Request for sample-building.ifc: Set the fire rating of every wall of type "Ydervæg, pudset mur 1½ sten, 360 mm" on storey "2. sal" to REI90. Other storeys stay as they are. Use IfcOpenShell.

First a look at what the model holds.

```python
import ifcopenshell
import ifcopenshell.util.element

model = ifcopenshell.open("sample-building.ifc")
print(model.schema)
storey = next(s for s in model.by_type("IfcBuildingStorey") if s.Name == "2. sal")
walls = [e for e in ifcopenshell.util.element.get_decomposition(storey) if e.is_a("IfcWall")]
seen = {}
for e in walls:
    element_type = ifcopenshell.util.element.get_type(e)
    key = (element_type.Name if element_type != e and element_type else None, ifcopenshell.util.element.get_pset(e, "Pset_WallCommon", "FireRating"))
    seen[key] = seen.get(key, 0) + 1
for (name, value), count in sorted(seen.items(), key=str):
    print(count, "x", name, "|", value)
```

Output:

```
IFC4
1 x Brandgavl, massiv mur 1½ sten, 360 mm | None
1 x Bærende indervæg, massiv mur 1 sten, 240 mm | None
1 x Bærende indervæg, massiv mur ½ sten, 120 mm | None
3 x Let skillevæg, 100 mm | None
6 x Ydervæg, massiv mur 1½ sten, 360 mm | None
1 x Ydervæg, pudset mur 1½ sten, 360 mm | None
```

```python
import ifcopenshell
import ifcopenshell.api.pset
import ifcopenshell.util.element

model = ifcopenshell.open("sample-building.ifc")

storey = next(s for s in model.by_type("IfcBuildingStorey") if s.Name == "2. sal")
walls = [e for e in ifcopenshell.util.element.get_decomposition(storey) if e.is_a("IfcWall")]

count = 0
for e in walls:
    element_type = ifcopenshell.util.element.get_type(e)
    if element_type in (None, e) or element_type.Name != "Ydervæg, pudset mur 1½ sten, 360 mm":
        continue
    found = ifcopenshell.util.element.get_pset(e, "Pset_WallCommon", should_inherit=False)
    if found:
        pset = model.by_id(found["id"])
        if len(ifcopenshell.util.element.get_elements_by_pset(pset)) > 1:
            pset = ifcopenshell.api.pset.unshare_pset(model, products=[e], pset=pset)[0]
    else:
        pset = ifcopenshell.api.pset.add_pset(model, product=e, name="Pset_WallCommon")
    ifcopenshell.api.pset.edit_pset(model, pset=pset, properties={"FireRating": "REI90"})
    count += 1

print(count, "walls updated")

model.write("sample-building_updated.ifc")
```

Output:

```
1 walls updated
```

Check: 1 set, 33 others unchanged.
